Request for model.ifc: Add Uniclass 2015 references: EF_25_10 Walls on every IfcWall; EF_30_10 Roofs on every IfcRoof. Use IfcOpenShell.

First a look at what the model holds.

```python
import ifcopenshell

model = ifcopenshell.open("model.ifc")
print(model.schema)
print("classifications:", [c.Name for c in model.by_type("IfcClassification")])
for ifc_class in ("IfcDoor", "IfcRoof", "IfcStair", "IfcWall", "IfcWindow"):
    print(ifc_class, len(model.by_type(ifc_class)))
```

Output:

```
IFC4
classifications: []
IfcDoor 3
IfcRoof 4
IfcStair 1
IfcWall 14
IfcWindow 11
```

```python
import ifcopenshell
import ifcopenshell.api.classification

model = ifcopenshell.open("model.ifc")

system = ifcopenshell.api.classification.add_classification(model, classification="Uniclass 2015")

codes = {
    "IfcWall": ("EF_25_10", "Walls"),
    "IfcRoof": ("EF_30_10", "Roofs"),
}
for ifc_class, (code, name) in codes.items():
    products = model.by_type(ifc_class)
    ifcopenshell.api.classification.add_reference(
        model, products=products, classification=system, identification=code, name=name
    )
    print(code, len(products))

model.write("model_updated.ifc")
```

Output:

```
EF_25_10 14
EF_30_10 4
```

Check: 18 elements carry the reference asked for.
